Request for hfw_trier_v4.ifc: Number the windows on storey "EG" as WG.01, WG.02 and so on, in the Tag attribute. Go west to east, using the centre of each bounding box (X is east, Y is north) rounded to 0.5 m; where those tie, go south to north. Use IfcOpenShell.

First a look at what the model holds.

```python
import ifcopenshell
import ifcopenshell.util.element
import ifcopenshell.util.placement

model = ifcopenshell.open("hfw_trier_v4.ifc")
print(model.schema)
storey = next(s for s in model.by_type("IfcBuildingStorey") if s.Name == "EG")
windows = [e for e in ifcopenshell.util.element.get_decomposition(storey) if e.is_a("IfcWindow")]
for e in sorted(windows, key=lambda e: e.id()):
    origin = ifcopenshell.util.placement.get_local_placement(e.ObjectPlacement)[:3, 3]
    print(e.id(), e.Tag, e.Name, origin.round(2) + 0.0, sep=" | ")
```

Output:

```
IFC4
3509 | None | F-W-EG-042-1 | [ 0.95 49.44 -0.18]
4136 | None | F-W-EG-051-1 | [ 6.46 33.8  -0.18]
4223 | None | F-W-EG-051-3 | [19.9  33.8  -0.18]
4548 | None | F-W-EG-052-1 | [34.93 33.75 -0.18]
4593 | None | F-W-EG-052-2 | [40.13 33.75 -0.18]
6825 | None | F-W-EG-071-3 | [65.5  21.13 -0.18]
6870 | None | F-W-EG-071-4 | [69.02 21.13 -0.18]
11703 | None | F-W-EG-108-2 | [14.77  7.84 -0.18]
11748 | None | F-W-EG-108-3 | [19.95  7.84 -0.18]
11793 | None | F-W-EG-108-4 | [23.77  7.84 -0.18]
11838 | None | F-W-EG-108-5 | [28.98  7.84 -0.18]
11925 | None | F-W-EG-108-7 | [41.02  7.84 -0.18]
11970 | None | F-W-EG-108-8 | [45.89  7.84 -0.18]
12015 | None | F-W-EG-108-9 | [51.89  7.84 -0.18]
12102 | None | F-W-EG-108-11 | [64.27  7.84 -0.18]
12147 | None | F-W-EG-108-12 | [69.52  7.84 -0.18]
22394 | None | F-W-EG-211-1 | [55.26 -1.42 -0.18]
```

```python
import ifcopenshell
import ifcopenshell.geom
import ifcopenshell.util.element
import ifcopenshell.util.shape

model = ifcopenshell.open("hfw_trier_v4.ifc")
settings = ifcopenshell.geom.settings()
settings.set("use-world-coords", True)


def centre(element):
    shape = ifcopenshell.geom.create_shape(settings, element)
    return ifcopenshell.util.shape.get_bbox_centroid(shape.geometry)


storey = next(s for s in model.by_type("IfcBuildingStorey") if s.Name == "EG")
windows = [e for e in ifcopenshell.util.element.get_decomposition(storey) if e.is_a("IfcWindow")]

# Insertion points can sit at a corner or the storey origin, so sort by the geometry (in metres).
centres = {e: centre(e) for e in windows}
windows.sort(key=lambda e: (round(centres[e][0] / 0.5), centres[e][1]))

for i, e in enumerate(windows, start=1):
    number = f"WG.{i:02d}"
    e.Tag = number
    print(e.id(), number)

model.write("hfw_trier_v4_edited.ifc")
```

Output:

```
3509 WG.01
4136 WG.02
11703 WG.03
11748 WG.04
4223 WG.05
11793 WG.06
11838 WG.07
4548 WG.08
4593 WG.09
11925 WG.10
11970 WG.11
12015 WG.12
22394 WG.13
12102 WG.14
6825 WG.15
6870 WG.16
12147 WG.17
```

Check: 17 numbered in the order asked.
